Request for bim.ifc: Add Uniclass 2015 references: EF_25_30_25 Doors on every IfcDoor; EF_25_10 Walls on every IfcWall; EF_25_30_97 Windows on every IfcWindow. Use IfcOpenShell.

First a look at what the model holds.

```python
import ifcopenshell

model = ifcopenshell.open("bim.ifc")
print(model.schema)
print("classifications:", [c.Name for c in model.by_type("IfcClassification")])
for ifc_class in ("IfcDoor", "IfcRoof", "IfcStair", "IfcWall", "IfcWindow"):
    print(ifc_class, len(model.by_type(ifc_class)))
```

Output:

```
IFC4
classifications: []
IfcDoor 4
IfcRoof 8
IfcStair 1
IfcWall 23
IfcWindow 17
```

```python
import ifcopenshell
import ifcopenshell.api.classification

model = ifcopenshell.open("bim.ifc")

system = ifcopenshell.api.classification.add_classification(model, classification="Uniclass 2015")

codes = {
    "IfcDoor": ("EF_25_30_25", "Doors"),
    "IfcWall": ("EF_25_10", "Walls"),
    "IfcWindow": ("EF_25_30_97", "Windows"),
}
for ifc_class, (code, name) in codes.items():
    products = model.by_type(ifc_class)
    ifcopenshell.api.classification.add_reference(
        model, products=products, classification=system, identification=code, name=name
    )
    print(code, len(products))

model.write("bim_edited.ifc")
```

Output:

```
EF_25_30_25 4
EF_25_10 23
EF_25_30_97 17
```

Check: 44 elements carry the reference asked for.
